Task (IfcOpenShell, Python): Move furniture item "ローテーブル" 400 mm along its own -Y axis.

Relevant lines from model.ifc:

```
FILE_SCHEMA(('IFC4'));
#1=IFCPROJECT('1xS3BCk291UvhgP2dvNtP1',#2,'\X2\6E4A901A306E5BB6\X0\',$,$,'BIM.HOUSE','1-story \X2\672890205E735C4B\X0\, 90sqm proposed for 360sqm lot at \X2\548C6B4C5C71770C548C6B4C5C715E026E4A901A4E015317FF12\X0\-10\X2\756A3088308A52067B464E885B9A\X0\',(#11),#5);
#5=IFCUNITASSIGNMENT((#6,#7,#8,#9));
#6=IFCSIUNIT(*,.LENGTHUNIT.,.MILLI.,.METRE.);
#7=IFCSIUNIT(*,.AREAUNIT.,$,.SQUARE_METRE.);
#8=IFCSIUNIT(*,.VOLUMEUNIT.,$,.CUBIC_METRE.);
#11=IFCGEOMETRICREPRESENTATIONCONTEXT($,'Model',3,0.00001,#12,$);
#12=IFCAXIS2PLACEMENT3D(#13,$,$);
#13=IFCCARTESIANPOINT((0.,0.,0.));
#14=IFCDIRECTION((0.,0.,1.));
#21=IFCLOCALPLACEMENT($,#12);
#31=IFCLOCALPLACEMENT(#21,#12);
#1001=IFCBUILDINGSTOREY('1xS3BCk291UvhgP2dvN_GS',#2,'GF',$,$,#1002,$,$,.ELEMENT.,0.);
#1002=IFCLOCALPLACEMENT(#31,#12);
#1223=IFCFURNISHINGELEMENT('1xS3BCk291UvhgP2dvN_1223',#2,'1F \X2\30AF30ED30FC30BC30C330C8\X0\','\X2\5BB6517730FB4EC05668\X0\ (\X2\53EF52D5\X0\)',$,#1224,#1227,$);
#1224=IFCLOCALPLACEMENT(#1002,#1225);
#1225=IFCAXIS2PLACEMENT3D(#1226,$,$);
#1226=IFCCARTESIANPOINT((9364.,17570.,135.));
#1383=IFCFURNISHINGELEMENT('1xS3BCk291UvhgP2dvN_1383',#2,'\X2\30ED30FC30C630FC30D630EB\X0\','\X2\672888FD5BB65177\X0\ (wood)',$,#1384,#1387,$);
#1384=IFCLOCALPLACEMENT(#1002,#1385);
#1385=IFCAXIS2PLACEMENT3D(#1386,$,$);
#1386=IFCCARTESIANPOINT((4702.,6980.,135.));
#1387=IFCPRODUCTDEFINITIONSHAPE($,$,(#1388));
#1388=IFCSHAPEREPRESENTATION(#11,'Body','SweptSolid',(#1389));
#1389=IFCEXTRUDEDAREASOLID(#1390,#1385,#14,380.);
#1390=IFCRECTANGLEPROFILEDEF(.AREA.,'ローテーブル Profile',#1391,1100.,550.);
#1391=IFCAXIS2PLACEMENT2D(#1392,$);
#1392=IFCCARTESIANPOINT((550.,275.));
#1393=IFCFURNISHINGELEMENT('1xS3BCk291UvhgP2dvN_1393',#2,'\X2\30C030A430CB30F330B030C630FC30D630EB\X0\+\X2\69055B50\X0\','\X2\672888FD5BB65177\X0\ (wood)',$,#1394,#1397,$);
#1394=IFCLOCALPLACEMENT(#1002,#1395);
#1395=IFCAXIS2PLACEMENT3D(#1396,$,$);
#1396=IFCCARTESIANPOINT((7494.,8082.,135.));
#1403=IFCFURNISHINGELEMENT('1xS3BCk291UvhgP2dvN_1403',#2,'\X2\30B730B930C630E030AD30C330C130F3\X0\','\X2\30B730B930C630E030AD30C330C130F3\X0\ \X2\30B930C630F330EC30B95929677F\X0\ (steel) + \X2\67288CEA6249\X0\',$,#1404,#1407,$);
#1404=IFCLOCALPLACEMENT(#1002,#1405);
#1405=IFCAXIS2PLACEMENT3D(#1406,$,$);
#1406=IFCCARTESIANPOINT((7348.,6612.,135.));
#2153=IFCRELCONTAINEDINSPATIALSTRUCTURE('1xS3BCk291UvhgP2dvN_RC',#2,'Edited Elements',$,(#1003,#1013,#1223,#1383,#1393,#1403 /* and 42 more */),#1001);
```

```python
import ifcopenshell
import ifcopenshell.api.geometry
import ifcopenshell.util.placement
import ifcopenshell.util.unit

model = ifcopenshell.open("model.ifc")
unit_scale = ifcopenshell.util.unit.calculate_unit_scale(model)

item = model.by_id(1383)
matrix = ifcopenshell.util.placement.get_local_placement(item.ObjectPlacement)
matrix[:3, 3] -= matrix[:3, 1] * 0.4 / unit_scale
ifcopenshell.api.geometry.edit_object_placement(model, product=item, matrix=matrix, is_si=False)

print(ifcopenshell.util.placement.get_local_placement(item.ObjectPlacement).round(3) + 0.0)

model.write("model_edited.ifc")
```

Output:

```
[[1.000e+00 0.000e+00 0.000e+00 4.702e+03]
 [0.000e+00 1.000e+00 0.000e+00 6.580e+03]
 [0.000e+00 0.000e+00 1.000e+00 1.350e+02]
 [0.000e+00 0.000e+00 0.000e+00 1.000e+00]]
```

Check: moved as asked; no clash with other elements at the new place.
